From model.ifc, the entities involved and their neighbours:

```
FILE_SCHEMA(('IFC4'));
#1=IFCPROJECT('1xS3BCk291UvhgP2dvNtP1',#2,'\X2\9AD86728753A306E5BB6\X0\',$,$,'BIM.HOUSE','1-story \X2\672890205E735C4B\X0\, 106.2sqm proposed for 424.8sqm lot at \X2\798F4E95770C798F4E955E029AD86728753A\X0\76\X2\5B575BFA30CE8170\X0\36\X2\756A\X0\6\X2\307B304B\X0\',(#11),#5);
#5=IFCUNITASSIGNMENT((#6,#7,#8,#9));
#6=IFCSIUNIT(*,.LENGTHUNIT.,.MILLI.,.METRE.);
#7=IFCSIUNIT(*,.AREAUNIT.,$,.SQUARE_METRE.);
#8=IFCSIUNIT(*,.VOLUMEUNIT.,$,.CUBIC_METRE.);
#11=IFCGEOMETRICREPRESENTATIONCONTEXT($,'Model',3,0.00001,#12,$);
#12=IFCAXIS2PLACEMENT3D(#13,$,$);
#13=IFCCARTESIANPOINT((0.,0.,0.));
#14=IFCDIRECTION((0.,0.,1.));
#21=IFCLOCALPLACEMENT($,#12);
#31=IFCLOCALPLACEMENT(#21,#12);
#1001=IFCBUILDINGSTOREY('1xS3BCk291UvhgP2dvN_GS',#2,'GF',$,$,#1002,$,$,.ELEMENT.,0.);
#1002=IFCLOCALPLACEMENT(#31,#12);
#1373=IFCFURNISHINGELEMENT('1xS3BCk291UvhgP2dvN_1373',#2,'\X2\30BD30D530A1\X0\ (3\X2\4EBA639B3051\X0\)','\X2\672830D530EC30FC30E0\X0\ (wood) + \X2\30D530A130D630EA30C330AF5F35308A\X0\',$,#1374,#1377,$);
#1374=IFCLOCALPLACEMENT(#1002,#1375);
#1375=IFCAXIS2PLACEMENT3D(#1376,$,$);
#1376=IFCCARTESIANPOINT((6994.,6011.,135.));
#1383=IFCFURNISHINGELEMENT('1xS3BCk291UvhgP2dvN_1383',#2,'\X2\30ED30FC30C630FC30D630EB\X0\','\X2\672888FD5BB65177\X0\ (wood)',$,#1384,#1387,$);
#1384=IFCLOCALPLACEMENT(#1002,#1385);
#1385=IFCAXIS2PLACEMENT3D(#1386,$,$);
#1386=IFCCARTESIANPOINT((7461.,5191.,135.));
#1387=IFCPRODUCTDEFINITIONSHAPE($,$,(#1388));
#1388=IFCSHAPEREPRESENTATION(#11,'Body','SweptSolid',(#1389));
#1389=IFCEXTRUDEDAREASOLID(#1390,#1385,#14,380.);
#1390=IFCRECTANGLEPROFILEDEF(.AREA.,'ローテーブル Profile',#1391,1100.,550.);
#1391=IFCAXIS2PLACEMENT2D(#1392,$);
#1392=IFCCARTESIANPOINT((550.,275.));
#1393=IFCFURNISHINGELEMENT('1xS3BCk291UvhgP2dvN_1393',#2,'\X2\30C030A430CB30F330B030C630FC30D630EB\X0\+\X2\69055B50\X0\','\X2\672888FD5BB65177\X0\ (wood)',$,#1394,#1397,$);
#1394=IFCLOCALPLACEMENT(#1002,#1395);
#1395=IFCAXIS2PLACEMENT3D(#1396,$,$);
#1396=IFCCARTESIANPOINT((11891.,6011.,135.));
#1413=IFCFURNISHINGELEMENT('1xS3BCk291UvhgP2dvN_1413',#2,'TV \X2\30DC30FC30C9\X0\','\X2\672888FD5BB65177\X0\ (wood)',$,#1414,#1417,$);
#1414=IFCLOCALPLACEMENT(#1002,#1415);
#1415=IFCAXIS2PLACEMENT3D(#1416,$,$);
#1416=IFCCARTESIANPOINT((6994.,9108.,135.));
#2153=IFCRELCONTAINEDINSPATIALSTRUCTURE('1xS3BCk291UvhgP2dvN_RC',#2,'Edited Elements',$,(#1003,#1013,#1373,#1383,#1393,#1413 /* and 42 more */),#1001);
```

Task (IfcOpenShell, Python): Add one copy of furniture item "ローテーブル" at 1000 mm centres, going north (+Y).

```python
import numpy as np
import ifcopenshell
import ifcopenshell.api.geometry
import ifcopenshell.api.root
import ifcopenshell.util.element
import ifcopenshell.util.placement

model = ifcopenshell.open("model.ifc")


def reuse_history(source, copy):
    """copy_class also copies each property set's owner history, people and application; keep the originals."""
    for rel in copy.IsDefinedBy:
        if rel.is_a("IfcRelDefinesByProperties") and (history := rel.RelatingPropertyDefinition.OwnerHistory):
            rel.RelatingPropertyDefinition.OwnerHistory = source.OwnerHistory
            ifcopenshell.util.element.remove_deep2(model, history)


source = model.by_guid("1xS3BCk291UvhgP2dvN_1383")
base = ifcopenshell.util.placement.get_local_placement(source.ObjectPlacement)
step = np.array([0.0, 1.0, 0.0]) * 1000.0

for i in range(1, 2):
    copy = ifcopenshell.api.root.copy_class(model, product=source)
    copy.Representation = ifcopenshell.util.element.copy_deep(
        model, source.Representation, exclude=["IfcGeometricRepresentationContext", "IfcRepresentationMap"]
    )
    reuse_history(source, copy)
    matrix = base.copy()
    matrix[:3, 3] += i * step
    print("added at", matrix[:3, 3].round(3) + 0.0)
    ifcopenshell.api.geometry.edit_object_placement(model, product=copy, matrix=matrix, is_si=False)

model.write("model_rev.ifc")
```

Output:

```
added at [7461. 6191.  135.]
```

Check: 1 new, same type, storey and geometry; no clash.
